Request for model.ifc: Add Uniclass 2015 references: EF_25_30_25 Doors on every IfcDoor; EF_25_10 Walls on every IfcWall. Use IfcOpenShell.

First a look at what the model holds.

```python
import ifcopenshell

model = ifcopenshell.open("model.ifc")
print(model.schema)
print("classifications:", [c.Name for c in model.by_type("IfcClassification")])
for ifc_class in ("IfcDoor", "IfcRoof", "IfcStair", "IfcWall", "IfcWindow"):
    print(ifc_class, len(model.by_type(ifc_class)))
```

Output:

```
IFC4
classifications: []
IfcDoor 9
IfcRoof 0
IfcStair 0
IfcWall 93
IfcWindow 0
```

```python
import ifcopenshell
import ifcopenshell.api.classification

model = ifcopenshell.open("model.ifc")

system = ifcopenshell.api.classification.add_classification(model, classification="Uniclass 2015")

codes = {
    "IfcDoor": ("EF_25_30_25", "Doors"),
    "IfcWall": ("EF_25_10", "Walls"),
}
for ifc_class, (code, name) in codes.items():
    products = model.by_type(ifc_class)
    ifcopenshell.api.classification.add_reference(
        model, products=products, classification=system, identification=code, name=name
    )
    print(code, len(products))

model.write("model_edited.ifc")
```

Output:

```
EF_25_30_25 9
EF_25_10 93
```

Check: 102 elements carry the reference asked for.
